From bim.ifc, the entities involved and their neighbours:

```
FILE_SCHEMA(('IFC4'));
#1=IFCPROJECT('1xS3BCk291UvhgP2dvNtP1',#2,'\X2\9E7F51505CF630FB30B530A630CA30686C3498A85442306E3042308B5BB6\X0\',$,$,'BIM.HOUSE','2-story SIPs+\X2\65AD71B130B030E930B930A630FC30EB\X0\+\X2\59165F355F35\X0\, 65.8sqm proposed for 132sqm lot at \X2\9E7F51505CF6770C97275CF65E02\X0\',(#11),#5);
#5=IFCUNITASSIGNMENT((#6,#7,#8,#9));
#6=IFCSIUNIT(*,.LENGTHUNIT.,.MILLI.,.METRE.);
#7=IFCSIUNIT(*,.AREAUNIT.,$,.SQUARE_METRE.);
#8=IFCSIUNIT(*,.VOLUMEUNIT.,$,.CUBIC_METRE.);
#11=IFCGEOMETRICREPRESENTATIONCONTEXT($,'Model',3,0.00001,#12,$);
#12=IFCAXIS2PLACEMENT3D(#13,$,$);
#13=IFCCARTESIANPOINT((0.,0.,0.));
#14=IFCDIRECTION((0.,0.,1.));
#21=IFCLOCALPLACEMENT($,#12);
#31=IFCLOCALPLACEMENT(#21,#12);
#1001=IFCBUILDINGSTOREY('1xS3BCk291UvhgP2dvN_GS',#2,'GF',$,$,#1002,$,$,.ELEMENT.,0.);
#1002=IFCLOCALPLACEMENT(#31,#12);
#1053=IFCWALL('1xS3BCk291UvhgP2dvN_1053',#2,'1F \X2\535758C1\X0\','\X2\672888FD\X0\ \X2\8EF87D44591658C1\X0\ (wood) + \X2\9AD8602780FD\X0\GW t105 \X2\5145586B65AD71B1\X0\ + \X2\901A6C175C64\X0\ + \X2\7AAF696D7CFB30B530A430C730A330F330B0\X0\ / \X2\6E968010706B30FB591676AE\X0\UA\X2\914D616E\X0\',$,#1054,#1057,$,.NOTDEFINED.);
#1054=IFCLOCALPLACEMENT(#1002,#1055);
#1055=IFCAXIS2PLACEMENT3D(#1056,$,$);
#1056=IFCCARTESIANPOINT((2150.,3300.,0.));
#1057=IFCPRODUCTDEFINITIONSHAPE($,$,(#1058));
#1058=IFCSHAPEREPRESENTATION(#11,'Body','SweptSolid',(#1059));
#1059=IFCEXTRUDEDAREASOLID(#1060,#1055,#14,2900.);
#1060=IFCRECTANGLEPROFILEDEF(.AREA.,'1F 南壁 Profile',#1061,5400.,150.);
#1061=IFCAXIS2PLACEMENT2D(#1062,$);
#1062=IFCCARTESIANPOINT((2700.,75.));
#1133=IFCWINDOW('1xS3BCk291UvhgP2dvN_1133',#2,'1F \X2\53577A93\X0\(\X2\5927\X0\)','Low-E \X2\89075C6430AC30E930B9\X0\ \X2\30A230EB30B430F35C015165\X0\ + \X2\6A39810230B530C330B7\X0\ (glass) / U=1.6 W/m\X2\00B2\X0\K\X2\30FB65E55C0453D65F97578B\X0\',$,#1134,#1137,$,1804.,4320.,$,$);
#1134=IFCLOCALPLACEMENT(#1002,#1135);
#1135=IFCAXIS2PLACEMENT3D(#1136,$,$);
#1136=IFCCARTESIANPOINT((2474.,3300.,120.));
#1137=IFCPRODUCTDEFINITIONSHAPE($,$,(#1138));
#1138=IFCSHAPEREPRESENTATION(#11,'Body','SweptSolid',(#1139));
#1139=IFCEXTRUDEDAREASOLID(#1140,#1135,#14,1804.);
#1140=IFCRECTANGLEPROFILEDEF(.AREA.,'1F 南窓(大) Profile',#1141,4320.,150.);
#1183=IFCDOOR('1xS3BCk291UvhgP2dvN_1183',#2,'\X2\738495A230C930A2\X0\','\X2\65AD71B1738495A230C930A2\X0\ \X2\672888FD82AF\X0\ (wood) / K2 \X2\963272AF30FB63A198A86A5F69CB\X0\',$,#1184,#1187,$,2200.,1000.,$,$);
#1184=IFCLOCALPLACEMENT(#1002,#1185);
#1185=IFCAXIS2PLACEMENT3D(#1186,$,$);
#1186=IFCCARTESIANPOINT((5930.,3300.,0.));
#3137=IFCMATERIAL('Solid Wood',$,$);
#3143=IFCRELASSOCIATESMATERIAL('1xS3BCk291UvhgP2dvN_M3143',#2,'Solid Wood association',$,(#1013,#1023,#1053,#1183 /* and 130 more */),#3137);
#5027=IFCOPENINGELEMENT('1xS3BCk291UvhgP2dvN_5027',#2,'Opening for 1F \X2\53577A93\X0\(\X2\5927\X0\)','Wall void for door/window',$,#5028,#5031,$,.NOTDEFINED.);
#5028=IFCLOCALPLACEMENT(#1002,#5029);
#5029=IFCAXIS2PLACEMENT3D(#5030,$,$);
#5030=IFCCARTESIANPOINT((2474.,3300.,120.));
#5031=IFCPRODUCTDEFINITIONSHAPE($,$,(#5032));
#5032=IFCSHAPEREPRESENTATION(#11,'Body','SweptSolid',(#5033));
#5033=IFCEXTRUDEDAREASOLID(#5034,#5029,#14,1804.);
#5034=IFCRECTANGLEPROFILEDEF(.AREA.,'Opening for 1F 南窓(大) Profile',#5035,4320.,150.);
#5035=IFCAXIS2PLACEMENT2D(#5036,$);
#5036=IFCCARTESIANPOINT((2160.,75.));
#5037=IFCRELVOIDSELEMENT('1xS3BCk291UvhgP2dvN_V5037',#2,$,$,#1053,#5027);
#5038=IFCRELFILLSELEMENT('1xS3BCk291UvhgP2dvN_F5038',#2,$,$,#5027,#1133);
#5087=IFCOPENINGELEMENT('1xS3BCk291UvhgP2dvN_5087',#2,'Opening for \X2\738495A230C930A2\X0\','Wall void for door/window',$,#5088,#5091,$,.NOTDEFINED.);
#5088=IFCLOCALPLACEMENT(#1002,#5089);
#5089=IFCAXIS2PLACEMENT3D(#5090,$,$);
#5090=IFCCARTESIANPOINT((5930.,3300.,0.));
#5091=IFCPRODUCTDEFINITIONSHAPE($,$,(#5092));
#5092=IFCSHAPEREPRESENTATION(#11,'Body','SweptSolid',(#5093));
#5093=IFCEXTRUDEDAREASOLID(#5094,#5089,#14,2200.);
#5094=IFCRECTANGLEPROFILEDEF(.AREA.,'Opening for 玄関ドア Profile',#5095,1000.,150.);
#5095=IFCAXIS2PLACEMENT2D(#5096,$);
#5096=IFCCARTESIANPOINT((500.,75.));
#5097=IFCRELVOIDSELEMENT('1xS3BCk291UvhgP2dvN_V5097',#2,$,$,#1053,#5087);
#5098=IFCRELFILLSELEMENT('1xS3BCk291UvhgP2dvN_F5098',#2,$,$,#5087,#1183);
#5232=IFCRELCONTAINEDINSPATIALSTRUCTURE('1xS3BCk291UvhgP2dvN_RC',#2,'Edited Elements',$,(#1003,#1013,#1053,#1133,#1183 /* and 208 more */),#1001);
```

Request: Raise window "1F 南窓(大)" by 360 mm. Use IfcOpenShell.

```python
import numpy as np
import ifcopenshell
import ifcopenshell.api.geometry
import ifcopenshell.util.placement
import ifcopenshell.util.unit

model = ifcopenshell.open("bim.ifc")
unit_scale = ifcopenshell.util.unit.calculate_unit_scale(model)

window = model.by_guid("1xS3BCk291UvhgP2dvN_1133")
opening = window.FillsVoids[0].RelatingOpeningElement
dz = 0.36 / unit_scale

shift = np.array([0.0, 0.0, dz])
# The window is not placed relative to its opening, so move both.
for product in (opening, window):
    matrix = ifcopenshell.util.placement.get_local_placement(product.ObjectPlacement)
    matrix[:3, 3] += shift
    ifcopenshell.api.geometry.edit_object_placement(model, product=product, matrix=matrix, is_si=False)

print(f"moved by {dz * unit_scale:+.3f} m")

model.write("bim-out.ifc")
```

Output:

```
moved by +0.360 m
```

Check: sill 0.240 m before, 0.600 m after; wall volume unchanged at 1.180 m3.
